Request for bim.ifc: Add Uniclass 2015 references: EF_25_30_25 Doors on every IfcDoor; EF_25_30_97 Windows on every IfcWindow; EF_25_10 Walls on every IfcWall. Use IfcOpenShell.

First a look at what the model holds.

```python
import ifcopenshell

model = ifcopenshell.open("bim.ifc")
print(model.schema)
print("classifications:", [c.Name for c in model.by_type("IfcClassification")])
for ifc_class in ("IfcDoor", "IfcRoof", "IfcStair", "IfcWall", "IfcWindow"):
    print(ifc_class, len(model.by_type(ifc_class)))
```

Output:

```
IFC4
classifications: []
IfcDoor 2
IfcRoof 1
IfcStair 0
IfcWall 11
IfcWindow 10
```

```python
import ifcopenshell
import ifcopenshell.api.classification

model = ifcopenshell.open("bim.ifc")

system = ifcopenshell.api.classification.add_classification(model, classification="Uniclass 2015")

codes = {
    "IfcDoor": ("EF_25_30_25", "Doors"),
    "IfcWindow": ("EF_25_30_97", "Windows"),
    "IfcWall": ("EF_25_10", "Walls"),
}
for ifc_class, (code, name) in codes.items():
    products = model.by_type(ifc_class)
    ifcopenshell.api.classification.add_reference(
        model, products=products, classification=system, identification=code, name=name
    )
    print(code, len(products))

model.write("bim_updated.ifc")
```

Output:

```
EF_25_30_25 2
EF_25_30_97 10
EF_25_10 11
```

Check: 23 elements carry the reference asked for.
